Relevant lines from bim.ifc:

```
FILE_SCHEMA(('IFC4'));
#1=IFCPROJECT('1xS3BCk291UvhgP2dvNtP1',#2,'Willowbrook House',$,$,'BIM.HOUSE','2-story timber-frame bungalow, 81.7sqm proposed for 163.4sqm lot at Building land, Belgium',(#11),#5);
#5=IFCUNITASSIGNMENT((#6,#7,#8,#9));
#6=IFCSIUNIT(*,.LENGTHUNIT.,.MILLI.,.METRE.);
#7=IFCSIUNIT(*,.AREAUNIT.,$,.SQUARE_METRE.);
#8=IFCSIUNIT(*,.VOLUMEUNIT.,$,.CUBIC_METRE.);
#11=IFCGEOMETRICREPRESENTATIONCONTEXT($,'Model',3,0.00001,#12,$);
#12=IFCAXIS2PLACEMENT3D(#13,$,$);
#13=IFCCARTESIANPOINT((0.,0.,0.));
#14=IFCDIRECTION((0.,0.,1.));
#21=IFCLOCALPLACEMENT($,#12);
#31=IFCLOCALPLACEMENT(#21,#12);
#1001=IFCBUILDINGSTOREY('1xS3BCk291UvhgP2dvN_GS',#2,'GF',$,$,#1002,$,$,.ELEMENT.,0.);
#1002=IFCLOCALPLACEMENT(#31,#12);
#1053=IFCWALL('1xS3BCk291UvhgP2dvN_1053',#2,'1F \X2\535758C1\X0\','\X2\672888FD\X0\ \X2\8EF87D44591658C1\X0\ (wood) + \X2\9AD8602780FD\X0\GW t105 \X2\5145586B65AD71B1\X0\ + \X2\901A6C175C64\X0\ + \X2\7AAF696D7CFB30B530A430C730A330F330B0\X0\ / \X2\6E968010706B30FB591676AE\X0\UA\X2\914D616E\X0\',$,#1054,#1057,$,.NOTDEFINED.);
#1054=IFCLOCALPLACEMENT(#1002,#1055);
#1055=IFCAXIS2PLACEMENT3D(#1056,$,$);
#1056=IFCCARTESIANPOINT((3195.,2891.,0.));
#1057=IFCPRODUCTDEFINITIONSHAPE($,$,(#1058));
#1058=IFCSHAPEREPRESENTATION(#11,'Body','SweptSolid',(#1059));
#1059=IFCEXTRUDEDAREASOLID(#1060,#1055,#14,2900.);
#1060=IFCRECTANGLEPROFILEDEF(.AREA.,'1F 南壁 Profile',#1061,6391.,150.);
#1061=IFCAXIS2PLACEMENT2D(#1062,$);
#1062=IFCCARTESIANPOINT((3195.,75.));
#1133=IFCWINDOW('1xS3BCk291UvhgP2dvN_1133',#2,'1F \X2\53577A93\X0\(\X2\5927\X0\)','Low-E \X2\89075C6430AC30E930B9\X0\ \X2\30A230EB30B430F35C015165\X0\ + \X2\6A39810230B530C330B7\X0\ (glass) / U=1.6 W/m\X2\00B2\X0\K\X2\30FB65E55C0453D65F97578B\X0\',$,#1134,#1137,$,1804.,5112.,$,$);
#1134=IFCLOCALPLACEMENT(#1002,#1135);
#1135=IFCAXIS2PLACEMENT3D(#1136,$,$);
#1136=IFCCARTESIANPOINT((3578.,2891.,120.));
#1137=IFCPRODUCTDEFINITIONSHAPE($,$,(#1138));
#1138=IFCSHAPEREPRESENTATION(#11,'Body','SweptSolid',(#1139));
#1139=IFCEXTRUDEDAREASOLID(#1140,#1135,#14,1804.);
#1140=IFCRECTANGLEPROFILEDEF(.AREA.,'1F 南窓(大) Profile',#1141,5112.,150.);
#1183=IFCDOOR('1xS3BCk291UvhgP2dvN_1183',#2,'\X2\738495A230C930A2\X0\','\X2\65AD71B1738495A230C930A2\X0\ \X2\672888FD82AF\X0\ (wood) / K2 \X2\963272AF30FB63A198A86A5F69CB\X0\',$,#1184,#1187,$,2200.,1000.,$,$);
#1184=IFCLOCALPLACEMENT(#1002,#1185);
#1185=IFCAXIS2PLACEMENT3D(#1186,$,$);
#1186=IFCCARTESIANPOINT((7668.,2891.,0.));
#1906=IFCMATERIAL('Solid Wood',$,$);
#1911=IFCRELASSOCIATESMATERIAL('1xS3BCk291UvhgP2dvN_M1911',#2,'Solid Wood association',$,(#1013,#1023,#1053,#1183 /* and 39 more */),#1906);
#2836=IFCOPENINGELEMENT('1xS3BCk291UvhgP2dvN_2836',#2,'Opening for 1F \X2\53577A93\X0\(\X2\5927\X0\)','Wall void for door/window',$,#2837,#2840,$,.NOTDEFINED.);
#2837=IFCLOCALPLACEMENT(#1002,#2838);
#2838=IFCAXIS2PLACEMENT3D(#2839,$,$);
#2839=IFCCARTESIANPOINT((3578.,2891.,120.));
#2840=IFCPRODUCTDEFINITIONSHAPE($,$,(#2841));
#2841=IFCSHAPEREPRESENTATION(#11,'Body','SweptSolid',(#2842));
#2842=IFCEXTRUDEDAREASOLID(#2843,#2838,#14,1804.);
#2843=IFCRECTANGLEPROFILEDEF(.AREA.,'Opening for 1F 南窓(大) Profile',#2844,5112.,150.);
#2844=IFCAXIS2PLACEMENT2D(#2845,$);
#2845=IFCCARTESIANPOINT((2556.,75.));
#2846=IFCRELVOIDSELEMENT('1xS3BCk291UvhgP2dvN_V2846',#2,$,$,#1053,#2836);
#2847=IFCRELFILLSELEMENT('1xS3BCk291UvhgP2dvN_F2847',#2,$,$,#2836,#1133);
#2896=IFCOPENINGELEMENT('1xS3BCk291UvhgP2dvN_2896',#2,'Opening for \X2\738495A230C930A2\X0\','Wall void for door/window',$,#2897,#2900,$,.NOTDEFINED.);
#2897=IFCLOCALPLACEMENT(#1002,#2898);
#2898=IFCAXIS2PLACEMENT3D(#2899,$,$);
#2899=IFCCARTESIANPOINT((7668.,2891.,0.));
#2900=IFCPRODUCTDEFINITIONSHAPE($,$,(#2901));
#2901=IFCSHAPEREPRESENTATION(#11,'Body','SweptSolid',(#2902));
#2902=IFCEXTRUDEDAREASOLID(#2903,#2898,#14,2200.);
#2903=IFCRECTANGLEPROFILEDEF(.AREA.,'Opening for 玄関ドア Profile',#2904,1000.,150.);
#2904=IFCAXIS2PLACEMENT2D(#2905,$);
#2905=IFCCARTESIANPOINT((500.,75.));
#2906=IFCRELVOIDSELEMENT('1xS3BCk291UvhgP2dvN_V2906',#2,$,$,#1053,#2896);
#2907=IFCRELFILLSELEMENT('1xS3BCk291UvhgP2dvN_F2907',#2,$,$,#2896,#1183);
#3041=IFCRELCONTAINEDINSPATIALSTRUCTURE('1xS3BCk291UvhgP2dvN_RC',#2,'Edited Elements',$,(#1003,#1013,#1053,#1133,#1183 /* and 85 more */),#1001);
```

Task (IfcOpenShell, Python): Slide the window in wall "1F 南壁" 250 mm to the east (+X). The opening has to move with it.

```python
import ifcopenshell
import ifcopenshell.api.geometry
import ifcopenshell.util.placement
import ifcopenshell.util.unit

model = ifcopenshell.open("bim.ifc")
unit_scale = ifcopenshell.util.unit.calculate_unit_scale(model)

window = model.by_id(1133)
opening = window.FillsVoids[0].RelatingOpeningElement
wall = opening.VoidsElements[0].RelatingBuildingElement

wall_matrix = ifcopenshell.util.placement.get_local_placement(wall.ObjectPlacement)
shift = wall_matrix[:3, 0] * 0.25 / unit_scale
before = ifcopenshell.util.placement.get_local_placement(window.ObjectPlacement)[:3, 3].copy()

# The window is not placed relative to its opening, so move both.
for product in (opening, window):
    matrix = ifcopenshell.util.placement.get_local_placement(product.ObjectPlacement)
    matrix[:3, 3] += shift
    ifcopenshell.api.geometry.edit_object_placement(model, product=product, matrix=matrix, is_si=False)

after = ifcopenshell.util.placement.get_local_placement(window.ObjectPlacement)[:3, 3]
print("window moved by", (after - before).round(3) + 0.0)

model.write("bim-out.ifc")
```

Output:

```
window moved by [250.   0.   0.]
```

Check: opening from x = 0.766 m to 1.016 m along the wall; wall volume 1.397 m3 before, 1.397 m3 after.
